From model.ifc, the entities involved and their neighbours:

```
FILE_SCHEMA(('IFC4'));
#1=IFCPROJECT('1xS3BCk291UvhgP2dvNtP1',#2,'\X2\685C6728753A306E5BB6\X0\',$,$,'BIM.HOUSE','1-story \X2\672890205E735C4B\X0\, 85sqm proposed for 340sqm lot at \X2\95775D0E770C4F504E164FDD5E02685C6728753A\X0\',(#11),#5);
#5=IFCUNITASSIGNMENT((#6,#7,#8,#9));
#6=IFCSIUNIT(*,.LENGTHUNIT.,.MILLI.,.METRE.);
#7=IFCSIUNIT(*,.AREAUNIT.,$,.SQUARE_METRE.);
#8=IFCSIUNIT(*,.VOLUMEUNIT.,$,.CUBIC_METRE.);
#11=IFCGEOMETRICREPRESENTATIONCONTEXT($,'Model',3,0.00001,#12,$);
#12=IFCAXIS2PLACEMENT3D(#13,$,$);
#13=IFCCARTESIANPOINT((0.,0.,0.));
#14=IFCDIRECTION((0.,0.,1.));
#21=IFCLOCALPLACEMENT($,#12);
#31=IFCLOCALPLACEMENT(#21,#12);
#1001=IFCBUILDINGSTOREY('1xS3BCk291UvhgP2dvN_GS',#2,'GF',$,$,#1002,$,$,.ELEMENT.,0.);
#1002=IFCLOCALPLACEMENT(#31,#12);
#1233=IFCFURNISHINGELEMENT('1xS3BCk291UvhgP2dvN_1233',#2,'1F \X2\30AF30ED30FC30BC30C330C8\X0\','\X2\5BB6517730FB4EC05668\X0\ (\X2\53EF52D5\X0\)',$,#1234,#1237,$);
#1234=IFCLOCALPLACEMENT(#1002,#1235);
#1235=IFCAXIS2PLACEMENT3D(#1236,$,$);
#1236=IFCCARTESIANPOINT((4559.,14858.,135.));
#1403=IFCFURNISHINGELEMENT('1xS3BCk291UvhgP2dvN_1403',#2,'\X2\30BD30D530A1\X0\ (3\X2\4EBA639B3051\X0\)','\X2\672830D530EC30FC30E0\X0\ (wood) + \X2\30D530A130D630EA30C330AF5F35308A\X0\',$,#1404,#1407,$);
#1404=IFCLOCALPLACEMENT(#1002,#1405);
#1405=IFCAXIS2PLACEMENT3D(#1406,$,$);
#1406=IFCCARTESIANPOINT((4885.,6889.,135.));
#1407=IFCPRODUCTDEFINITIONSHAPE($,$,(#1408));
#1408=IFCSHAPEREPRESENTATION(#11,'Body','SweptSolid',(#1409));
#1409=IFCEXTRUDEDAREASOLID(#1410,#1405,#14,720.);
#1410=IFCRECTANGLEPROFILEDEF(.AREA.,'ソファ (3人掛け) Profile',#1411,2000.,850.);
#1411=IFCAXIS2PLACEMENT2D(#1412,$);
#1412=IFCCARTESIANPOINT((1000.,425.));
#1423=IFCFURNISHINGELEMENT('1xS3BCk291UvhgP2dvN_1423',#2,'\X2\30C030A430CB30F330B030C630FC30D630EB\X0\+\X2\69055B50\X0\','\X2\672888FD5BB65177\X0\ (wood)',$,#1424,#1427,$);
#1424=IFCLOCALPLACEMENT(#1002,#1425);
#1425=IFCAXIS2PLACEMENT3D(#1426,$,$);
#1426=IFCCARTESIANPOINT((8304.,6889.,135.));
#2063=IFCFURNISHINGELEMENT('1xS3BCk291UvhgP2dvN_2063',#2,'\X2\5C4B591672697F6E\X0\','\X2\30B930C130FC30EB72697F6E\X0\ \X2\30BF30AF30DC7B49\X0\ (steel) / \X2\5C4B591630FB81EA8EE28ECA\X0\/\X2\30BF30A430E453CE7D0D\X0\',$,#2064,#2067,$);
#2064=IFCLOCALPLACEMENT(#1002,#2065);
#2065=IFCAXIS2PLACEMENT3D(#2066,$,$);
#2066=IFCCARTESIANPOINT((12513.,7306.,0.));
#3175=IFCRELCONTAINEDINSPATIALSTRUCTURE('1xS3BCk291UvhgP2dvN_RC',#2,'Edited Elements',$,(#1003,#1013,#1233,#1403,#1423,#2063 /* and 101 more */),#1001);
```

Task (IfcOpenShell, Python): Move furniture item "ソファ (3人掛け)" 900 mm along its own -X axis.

```python
import ifcopenshell
import ifcopenshell.api.geometry
import ifcopenshell.util.placement
import ifcopenshell.util.unit

model = ifcopenshell.open("model.ifc")
unit_scale = ifcopenshell.util.unit.calculate_unit_scale(model)

item = model.by_id(1403)
matrix = ifcopenshell.util.placement.get_local_placement(item.ObjectPlacement)
matrix[:3, 3] -= matrix[:3, 0] * 0.9 / unit_scale
ifcopenshell.api.geometry.edit_object_placement(model, product=item, matrix=matrix, is_si=False)

print(ifcopenshell.util.placement.get_local_placement(item.ObjectPlacement).round(3) + 0.0)

model.write("model_updated.ifc")
```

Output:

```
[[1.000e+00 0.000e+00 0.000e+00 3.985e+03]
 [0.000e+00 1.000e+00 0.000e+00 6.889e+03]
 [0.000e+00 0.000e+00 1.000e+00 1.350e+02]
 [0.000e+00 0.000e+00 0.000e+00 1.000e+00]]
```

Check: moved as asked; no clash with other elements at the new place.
